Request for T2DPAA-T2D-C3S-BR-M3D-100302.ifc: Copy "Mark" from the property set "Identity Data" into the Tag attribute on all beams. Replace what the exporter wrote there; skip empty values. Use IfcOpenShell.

First a look at what the model holds.

```python
import ifcopenshell
import ifcopenshell.util.element

model = ifcopenshell.open("T2DPAA-T2D-C3S-BR-M3D-100302.ifc")
print(model.schema)
beams = model.by_type("IfcBeam")
print(len(beams), "beams")
for e in beams[:8]:
    source = ifcopenshell.util.element.get_pset(e, "Identity Data", "Mark")
    target = e.Tag
    print(e.id(), repr(source), repr(target), sep=" | ")
```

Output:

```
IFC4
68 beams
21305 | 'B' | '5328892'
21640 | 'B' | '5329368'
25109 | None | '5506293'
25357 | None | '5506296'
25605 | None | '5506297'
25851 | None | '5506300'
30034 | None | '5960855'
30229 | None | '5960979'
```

```python
import ifcopenshell
import ifcopenshell.util.element

model = ifcopenshell.open("T2DPAA-T2D-C3S-BR-M3D-100302.ifc")

count = 0
for e in model.by_type("IfcBeam"):
    value = ifcopenshell.util.element.get_pset(e, "Identity Data", "Mark")
    current = e.Tag
    if not value or not value.strip() or current == value:
        continue
    e.Tag = value
    count += 1

print(count, "beams updated")

model.write("T2DPAA-T2D-C3S-BR-M3D-100302-out.ifc")
```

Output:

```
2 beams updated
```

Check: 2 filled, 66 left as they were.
